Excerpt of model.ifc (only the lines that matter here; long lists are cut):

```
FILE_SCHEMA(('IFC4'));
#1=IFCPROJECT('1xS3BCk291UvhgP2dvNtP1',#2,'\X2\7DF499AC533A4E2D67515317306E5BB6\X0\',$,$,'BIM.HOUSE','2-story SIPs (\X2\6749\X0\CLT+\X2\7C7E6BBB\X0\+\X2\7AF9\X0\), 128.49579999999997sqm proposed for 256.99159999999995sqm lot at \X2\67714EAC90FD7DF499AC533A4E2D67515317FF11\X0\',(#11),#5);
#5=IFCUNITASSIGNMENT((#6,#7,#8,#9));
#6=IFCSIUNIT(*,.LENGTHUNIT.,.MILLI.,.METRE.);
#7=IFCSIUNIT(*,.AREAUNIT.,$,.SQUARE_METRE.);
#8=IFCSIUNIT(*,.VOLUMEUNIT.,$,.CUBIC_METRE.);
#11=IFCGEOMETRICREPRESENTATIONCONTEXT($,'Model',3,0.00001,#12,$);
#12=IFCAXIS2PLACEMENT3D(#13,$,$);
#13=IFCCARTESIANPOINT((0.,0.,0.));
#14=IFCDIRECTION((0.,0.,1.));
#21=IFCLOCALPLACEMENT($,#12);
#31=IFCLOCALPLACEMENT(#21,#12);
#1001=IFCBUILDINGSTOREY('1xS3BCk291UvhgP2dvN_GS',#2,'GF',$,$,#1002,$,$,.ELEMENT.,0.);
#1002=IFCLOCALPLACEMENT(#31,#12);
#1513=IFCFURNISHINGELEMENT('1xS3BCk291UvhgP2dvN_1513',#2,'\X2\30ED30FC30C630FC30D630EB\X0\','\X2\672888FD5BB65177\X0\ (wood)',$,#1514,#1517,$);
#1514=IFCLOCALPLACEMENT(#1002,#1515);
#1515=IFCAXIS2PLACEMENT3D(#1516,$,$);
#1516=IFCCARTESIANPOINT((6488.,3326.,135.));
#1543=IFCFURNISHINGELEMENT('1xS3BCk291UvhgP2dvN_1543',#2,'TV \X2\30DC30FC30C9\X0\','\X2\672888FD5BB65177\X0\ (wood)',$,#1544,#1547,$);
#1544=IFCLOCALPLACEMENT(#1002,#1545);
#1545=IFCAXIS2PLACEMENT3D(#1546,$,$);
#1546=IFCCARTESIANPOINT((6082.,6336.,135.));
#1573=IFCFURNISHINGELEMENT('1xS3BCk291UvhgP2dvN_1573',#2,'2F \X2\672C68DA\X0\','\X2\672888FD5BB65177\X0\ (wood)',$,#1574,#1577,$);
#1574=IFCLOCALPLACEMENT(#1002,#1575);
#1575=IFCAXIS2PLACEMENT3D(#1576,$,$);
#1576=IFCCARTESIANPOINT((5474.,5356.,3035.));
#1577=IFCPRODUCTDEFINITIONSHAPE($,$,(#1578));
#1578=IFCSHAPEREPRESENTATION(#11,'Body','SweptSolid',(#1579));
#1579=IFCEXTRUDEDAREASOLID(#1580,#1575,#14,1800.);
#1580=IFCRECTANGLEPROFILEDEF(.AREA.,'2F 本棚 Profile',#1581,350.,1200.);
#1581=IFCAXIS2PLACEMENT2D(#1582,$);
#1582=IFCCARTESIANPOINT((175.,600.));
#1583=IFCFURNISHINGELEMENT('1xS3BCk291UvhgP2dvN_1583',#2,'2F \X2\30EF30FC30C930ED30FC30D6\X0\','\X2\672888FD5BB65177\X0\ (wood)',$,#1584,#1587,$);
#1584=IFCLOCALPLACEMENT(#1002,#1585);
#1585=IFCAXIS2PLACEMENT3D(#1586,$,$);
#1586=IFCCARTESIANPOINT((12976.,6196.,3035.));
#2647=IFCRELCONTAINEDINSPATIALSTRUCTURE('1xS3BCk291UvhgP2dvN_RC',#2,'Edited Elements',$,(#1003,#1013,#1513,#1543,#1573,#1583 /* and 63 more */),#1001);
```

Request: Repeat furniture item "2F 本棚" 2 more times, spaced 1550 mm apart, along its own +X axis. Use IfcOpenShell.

```python
import ifcopenshell
import ifcopenshell.api.geometry
import ifcopenshell.api.root
import ifcopenshell.util.element
import ifcopenshell.util.placement
import ifcopenshell.util.unit

model = ifcopenshell.open("model.ifc")
unit_scale = ifcopenshell.util.unit.calculate_unit_scale(model)


def reuse_history(source, copy):
    """copy_class also copies each property set's owner history, people and application; keep the originals."""
    for rel in copy.IsDefinedBy:
        if rel.is_a("IfcRelDefinesByProperties") and (history := rel.RelatingPropertyDefinition.OwnerHistory):
            rel.RelatingPropertyDefinition.OwnerHistory = source.OwnerHistory
            ifcopenshell.util.element.remove_deep2(model, history)


source = model.by_guid("1xS3BCk291UvhgP2dvN_1573")
base = ifcopenshell.util.placement.get_local_placement(source.ObjectPlacement)
step = base[:3, 0] * 1.55 / unit_scale

for i in range(1, 3):
    copy = ifcopenshell.api.root.copy_class(model, product=source)
    copy.Representation = ifcopenshell.util.element.copy_deep(
        model, source.Representation, exclude=["IfcGeometricRepresentationContext", "IfcRepresentationMap"]
    )
    reuse_history(source, copy)
    matrix = base.copy()
    matrix[:3, 3] += i * step
    print("added at", matrix[:3, 3].round(3) + 0.0)
    ifcopenshell.api.geometry.edit_object_placement(model, product=copy, matrix=matrix, is_si=False)

model.write("model_edited.ifc")
```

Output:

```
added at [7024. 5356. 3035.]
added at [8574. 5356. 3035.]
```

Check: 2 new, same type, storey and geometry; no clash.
